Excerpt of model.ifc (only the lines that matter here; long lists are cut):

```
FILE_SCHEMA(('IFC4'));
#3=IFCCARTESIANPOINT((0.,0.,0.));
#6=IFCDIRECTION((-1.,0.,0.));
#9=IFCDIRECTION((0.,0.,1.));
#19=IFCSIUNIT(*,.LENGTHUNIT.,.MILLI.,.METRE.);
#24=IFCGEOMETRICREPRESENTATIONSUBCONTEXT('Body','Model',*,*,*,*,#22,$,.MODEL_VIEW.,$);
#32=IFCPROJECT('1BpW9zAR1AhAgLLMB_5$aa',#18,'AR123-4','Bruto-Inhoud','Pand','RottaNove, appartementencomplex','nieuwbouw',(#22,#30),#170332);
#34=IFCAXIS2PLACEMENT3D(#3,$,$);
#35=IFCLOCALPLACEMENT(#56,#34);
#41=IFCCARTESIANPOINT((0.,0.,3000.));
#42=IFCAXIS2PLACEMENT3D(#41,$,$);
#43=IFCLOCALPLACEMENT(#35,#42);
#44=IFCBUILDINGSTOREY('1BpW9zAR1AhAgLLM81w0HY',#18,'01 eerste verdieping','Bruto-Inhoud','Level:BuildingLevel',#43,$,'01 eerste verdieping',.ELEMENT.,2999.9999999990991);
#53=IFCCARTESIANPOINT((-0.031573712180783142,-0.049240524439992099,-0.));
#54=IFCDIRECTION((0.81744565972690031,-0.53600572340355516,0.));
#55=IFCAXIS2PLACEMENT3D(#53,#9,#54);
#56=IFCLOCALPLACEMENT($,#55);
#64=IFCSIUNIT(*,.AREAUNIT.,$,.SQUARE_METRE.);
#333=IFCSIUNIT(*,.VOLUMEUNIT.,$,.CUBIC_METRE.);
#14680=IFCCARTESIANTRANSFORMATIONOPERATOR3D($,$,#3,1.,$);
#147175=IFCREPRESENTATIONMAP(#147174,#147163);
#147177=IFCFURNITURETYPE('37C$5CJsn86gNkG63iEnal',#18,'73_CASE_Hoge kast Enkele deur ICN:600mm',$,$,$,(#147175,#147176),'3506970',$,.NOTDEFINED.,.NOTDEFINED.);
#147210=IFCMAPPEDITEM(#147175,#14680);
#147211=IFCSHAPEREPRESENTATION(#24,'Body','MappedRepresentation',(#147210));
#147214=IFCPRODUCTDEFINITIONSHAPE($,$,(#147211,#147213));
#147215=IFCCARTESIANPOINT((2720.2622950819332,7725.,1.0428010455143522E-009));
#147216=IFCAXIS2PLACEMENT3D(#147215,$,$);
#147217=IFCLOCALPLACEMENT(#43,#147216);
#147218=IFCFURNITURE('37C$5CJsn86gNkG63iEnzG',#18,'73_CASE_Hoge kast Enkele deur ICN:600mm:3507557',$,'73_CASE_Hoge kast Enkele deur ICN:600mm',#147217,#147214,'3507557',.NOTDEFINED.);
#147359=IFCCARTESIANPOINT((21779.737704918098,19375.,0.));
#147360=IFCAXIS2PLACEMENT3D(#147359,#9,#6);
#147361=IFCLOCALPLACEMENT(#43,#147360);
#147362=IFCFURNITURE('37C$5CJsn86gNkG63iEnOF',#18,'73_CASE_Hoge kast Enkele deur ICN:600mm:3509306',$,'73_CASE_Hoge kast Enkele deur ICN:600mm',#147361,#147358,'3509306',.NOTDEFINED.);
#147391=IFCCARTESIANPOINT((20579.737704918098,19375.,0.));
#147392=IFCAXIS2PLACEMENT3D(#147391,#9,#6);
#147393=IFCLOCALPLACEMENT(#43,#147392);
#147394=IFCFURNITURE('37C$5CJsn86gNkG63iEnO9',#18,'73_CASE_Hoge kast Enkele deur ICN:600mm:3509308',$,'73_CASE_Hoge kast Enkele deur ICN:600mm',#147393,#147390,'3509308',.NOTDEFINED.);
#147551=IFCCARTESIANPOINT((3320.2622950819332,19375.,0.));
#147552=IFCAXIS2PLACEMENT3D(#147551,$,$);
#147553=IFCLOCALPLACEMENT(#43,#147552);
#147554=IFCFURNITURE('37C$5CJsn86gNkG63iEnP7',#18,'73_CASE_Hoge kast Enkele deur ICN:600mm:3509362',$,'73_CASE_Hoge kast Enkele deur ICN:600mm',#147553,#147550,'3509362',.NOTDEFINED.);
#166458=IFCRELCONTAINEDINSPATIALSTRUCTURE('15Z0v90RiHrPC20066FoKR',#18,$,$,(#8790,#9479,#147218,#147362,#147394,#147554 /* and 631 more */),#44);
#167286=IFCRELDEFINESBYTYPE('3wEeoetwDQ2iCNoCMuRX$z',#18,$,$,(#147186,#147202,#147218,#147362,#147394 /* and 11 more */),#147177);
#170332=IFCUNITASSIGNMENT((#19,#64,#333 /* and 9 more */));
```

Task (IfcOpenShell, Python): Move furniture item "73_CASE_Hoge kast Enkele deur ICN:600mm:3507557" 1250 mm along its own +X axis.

```python
import ifcopenshell
import ifcopenshell.api.geometry
import ifcopenshell.util.placement

model = ifcopenshell.open("model.ifc")

item = model.by_guid("37C$5CJsn86gNkG63iEnzG")
matrix = ifcopenshell.util.placement.get_local_placement(item.ObjectPlacement)
matrix[:3, 3] += matrix[:3, 0] * 1250.0
ifcopenshell.api.geometry.edit_object_placement(model, product=item, matrix=matrix, is_si=False)

print(ifcopenshell.util.placement.get_local_placement(item.ObjectPlacement).round(3) + 0.0)

model.write("model_updated.ifc")
```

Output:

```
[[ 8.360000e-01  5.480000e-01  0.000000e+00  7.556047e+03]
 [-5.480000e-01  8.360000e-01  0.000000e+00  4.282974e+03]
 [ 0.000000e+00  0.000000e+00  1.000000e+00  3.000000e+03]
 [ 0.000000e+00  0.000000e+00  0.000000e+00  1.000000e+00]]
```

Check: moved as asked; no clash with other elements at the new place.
